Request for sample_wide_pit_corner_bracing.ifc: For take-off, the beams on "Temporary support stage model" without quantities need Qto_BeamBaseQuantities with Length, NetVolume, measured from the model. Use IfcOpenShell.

First a look at what the model holds.

```python
import ifcopenshell
import ifcopenshell.util.element
import ifcopenshell.util.unit

model = ifcopenshell.open("sample_wide_pit_corner_bracing.ifc")
print(model.schema)
for unit_type in ("LENGTHUNIT", "AREAUNIT", "VOLUMEUNIT"):
    print(unit_type, ifcopenshell.util.unit.calculate_unit_scale(model, unit_type))
storey = next(s for s in model.by_type("IfcBuildingStorey") if s.Name == "Temporary support stage model")
beams = [e for e in ifcopenshell.util.element.get_decomposition(storey) if e.is_a("IfcBeam")]
for e in sorted(beams, key=lambda e: e.id()):
    print(e.id(), e.is_a(), e.Name, list(ifcopenshell.util.element.get_psets(e, qtos_only=True)), sep=" | ")
```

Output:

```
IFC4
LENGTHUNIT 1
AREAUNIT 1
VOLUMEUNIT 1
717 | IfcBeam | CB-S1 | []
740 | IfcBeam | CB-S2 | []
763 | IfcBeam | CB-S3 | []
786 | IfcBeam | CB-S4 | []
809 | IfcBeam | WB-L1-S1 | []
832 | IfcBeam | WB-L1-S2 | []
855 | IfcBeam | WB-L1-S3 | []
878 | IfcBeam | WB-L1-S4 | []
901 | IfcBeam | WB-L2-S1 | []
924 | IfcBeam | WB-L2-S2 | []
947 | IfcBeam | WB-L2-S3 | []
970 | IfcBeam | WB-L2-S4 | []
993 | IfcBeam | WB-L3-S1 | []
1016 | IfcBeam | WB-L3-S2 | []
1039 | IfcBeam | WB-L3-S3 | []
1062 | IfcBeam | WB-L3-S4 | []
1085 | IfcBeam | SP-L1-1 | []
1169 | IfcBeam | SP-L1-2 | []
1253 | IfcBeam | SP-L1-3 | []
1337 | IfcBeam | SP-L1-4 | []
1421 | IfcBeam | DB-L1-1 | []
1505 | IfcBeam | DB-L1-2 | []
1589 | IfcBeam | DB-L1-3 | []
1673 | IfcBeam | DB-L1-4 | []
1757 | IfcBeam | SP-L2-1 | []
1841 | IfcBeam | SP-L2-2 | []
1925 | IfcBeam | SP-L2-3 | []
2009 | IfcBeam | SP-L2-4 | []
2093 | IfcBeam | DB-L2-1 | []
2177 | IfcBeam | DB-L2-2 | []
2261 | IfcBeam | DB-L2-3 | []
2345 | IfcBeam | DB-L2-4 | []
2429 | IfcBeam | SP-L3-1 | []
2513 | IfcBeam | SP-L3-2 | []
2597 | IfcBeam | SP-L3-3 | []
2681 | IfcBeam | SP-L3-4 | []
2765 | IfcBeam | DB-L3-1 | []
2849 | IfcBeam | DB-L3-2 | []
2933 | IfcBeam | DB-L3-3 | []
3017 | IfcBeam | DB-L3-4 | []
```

```python
import ifcopenshell
import ifcopenshell.api.pset
import ifcopenshell.geom
import ifcopenshell.util.element
import ifcopenshell.util.shape
import ifcopenshell.util.unit

model = ifcopenshell.open("sample_wide_pit_corner_bracing.ifc")
unit_scale = ifcopenshell.util.unit.calculate_unit_scale(model)
volume_scale = ifcopenshell.util.unit.calculate_unit_scale(model, "VOLUMEUNIT")
settings = ifcopenshell.geom.settings()

storey = next(s for s in model.by_type("IfcBuildingStorey") if s.Name == "Temporary support stage model")
beams = [e for e in ifcopenshell.util.element.get_decomposition(storey) if e.is_a("IfcBeam")]

for e in sorted(beams, key=lambda e: e.id()):
    if ifcopenshell.util.element.get_psets(e, qtos_only=True, should_inherit=False):
        continue
    # Geometry comes back in metres, in the element's own axes.
    shape = ifcopenshell.geom.create_shape(settings, e)
    values = {
        "Length": ifcopenshell.util.shape.get_max_xyz(shape.geometry) / unit_scale,
        "NetVolume": ifcopenshell.util.shape.get_volume(shape.geometry) / volume_scale,
    }
    qto = ifcopenshell.api.pset.add_qto(model, product=e, name="Qto_BeamBaseQuantities")
    ifcopenshell.api.pset.edit_qto(model, qto=qto, properties=values)
    print(e.id(), {k: round(v, 3) for k, v in values.items()})

model.write("sample_wide_pit_corner_bracing_v2.ifc")
```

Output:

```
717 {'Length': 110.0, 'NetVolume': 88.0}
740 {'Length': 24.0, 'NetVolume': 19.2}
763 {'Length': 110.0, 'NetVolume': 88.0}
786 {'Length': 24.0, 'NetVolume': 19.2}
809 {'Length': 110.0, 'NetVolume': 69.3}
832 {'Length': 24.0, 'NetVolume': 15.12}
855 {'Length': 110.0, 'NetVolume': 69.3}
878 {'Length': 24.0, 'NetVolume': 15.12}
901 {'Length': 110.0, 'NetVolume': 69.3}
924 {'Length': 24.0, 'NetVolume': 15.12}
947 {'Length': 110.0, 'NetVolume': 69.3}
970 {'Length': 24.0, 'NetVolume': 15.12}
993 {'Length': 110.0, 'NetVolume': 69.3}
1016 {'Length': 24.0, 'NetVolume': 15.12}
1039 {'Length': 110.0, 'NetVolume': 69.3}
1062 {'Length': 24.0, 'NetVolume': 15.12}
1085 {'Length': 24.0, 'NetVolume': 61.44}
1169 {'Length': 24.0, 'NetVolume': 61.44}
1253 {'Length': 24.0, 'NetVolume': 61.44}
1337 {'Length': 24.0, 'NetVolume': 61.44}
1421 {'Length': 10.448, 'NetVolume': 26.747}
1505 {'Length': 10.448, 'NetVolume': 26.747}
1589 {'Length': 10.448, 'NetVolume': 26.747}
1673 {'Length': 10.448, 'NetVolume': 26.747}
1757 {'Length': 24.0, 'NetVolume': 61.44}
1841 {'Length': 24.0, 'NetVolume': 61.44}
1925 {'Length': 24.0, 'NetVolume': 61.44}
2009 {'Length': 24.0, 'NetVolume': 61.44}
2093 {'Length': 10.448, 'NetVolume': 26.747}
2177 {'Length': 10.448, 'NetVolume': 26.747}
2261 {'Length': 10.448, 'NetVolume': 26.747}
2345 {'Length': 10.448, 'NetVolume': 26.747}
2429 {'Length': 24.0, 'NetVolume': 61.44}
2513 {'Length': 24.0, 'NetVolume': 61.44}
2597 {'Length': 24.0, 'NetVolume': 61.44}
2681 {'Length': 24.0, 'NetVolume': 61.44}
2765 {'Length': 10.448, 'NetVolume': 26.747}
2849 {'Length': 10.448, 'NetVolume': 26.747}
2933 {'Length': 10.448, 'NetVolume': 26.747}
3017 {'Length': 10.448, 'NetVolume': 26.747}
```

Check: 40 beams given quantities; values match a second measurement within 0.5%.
